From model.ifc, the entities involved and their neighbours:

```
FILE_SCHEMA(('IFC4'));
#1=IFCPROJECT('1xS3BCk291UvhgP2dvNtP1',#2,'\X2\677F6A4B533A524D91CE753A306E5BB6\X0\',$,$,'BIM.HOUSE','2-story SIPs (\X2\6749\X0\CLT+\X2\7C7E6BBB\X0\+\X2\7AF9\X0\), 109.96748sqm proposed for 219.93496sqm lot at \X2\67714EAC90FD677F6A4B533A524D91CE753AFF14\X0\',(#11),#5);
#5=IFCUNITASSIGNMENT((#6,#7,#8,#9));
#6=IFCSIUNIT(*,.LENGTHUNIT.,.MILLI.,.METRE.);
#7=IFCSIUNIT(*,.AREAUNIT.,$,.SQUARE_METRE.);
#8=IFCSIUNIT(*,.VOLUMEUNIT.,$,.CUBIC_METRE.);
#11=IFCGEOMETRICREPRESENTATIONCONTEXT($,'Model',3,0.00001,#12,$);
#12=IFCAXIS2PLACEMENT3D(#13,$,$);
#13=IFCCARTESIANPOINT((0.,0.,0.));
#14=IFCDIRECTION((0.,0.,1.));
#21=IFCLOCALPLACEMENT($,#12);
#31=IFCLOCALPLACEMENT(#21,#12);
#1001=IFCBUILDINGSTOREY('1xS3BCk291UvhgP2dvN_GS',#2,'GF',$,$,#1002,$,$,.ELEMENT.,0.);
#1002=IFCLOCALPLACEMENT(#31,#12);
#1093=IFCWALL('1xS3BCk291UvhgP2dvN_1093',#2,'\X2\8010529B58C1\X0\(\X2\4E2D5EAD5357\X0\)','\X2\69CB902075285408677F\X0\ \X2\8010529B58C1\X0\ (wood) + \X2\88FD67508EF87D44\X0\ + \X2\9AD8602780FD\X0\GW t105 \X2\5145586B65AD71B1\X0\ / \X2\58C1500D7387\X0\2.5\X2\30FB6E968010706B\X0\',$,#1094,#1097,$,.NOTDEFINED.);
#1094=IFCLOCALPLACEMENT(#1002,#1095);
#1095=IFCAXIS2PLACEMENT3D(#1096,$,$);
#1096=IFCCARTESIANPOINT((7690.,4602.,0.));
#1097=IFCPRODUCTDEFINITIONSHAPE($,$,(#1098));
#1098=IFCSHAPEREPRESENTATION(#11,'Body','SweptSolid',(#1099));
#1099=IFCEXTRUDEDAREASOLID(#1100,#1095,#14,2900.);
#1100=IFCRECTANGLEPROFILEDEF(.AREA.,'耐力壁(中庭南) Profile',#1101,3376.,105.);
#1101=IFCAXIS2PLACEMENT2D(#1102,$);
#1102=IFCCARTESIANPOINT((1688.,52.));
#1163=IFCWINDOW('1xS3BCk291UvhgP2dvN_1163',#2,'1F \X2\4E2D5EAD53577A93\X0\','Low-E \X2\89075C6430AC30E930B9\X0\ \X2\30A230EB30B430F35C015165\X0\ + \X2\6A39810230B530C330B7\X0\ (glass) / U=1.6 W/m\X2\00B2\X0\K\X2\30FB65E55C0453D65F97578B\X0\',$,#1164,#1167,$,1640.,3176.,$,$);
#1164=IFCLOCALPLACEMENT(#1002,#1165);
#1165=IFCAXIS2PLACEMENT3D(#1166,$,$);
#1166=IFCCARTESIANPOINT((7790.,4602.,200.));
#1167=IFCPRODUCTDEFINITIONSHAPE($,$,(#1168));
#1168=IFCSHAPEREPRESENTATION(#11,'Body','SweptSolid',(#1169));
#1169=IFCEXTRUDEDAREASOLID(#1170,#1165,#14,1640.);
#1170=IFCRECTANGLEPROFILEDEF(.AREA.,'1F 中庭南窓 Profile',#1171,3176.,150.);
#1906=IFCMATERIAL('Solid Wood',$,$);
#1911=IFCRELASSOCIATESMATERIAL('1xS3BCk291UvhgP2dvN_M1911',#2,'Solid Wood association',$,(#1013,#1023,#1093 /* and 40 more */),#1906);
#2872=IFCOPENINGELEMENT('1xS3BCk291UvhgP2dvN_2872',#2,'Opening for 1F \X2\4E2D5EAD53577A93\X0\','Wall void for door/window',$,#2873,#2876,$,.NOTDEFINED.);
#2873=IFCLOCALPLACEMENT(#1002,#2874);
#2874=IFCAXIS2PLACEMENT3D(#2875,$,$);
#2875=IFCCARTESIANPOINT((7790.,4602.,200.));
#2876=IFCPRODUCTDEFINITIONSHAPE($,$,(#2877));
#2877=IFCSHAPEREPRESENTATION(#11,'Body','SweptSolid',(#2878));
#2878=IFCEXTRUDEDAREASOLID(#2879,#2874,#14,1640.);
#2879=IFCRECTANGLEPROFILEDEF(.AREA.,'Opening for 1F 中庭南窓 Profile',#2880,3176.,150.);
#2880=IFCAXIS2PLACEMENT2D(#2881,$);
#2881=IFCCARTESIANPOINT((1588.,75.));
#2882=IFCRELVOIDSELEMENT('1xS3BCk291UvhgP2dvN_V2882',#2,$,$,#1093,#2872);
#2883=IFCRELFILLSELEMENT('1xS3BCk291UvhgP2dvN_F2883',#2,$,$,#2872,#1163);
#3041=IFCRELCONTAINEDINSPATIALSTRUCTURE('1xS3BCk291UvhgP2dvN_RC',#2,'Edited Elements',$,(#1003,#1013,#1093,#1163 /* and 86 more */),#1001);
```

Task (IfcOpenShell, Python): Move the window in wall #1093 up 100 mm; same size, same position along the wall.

```python
import numpy as np
import ifcopenshell
import ifcopenshell.api.geometry
import ifcopenshell.util.placement
import ifcopenshell.util.unit

model = ifcopenshell.open("model.ifc")
unit_scale = ifcopenshell.util.unit.calculate_unit_scale(model)

window = model.by_guid("1xS3BCk291UvhgP2dvN_1163")
opening = window.FillsVoids[0].RelatingOpeningElement
dz = 0.1 / unit_scale

shift = np.array([0.0, 0.0, dz])
# The window is not placed relative to its opening, so move both.
for product in (opening, window):
    matrix = ifcopenshell.util.placement.get_local_placement(product.ObjectPlacement)
    matrix[:3, 3] += shift
    ifcopenshell.api.geometry.edit_object_placement(model, product=product, matrix=matrix, is_si=False)

print(f"moved by {dz * unit_scale:+.3f} m")

model.write("model_rev.ifc")
```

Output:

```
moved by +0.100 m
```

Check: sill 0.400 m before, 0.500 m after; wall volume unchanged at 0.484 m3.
